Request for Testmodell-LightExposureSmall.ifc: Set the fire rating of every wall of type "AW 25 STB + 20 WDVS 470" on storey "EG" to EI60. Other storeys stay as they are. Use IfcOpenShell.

First a look at what the model holds.

```python
import ifcopenshell
import ifcopenshell.util.element

model = ifcopenshell.open("Testmodell-LightExposureSmall.ifc")
print(model.schema)
storey = next(s for s in model.by_type("IfcBuildingStorey") if s.Name == "EG")
walls = [e for e in ifcopenshell.util.element.get_decomposition(storey) if e.is_a("IfcWall")]
seen = {}
for e in walls:
    element_type = ifcopenshell.util.element.get_type(e)
    key = (element_type.Name if element_type != e and element_type else None, ifcopenshell.util.element.get_pset(e, "Pset_WallCommon", "FireRating"))
    seen[key] = seen.get(key, 0) + 1
for (name, value), count in sorted(seen.items(), key=str):
    print(count, "x", name, "|", value)
```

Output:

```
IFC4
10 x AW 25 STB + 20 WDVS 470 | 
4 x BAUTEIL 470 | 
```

```python
import ifcopenshell
import ifcopenshell.api.pset
import ifcopenshell.util.element

model = ifcopenshell.open("Testmodell-LightExposureSmall.ifc")

storey = next(s for s in model.by_type("IfcBuildingStorey") if s.Name == "EG")
walls = [e for e in ifcopenshell.util.element.get_decomposition(storey) if e.is_a("IfcWall")]

count = 0
for e in walls:
    element_type = ifcopenshell.util.element.get_type(e)
    if element_type in (None, e) or element_type.Name != "AW 25 STB + 20 WDVS 470":
        continue
    # add_pset returns the element's existing set when there is one.
    pset = ifcopenshell.api.pset.add_pset(model, product=e, name="Pset_WallCommon")
    ifcopenshell.api.pset.edit_pset(model, pset=pset, properties={"FireRating": "EI60"})
    count += 1

print(count, "walls updated")

model.write("Testmodell-LightExposureSmall_updated.ifc")
```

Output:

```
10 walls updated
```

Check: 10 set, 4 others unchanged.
